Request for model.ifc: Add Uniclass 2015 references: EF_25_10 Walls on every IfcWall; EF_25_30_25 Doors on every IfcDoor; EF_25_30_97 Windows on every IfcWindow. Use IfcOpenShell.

First a look at what the model holds.

```python
import ifcopenshell

model = ifcopenshell.open("model.ifc")
print(model.schema)
print("classifications:", [c.Name for c in model.by_type("IfcClassification")])
for ifc_class in ("IfcDoor", "IfcRoof", "IfcStair", "IfcWall", "IfcWindow"):
    print(ifc_class, len(model.by_type(ifc_class)))
```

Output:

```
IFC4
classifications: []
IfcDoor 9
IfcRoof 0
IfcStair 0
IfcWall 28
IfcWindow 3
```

```python
import ifcopenshell
import ifcopenshell.api.classification

model = ifcopenshell.open("model.ifc")

system = ifcopenshell.api.classification.add_classification(model, classification="Uniclass 2015")

codes = {
    "IfcWall": ("EF_25_10", "Walls"),
    "IfcDoor": ("EF_25_30_25", "Doors"),
    "IfcWindow": ("EF_25_30_97", "Windows"),
}
for ifc_class, (code, name) in codes.items():
    products = model.by_type(ifc_class)
    ifcopenshell.api.classification.add_reference(
        model, products=products, classification=system, identification=code, name=name
    )
    print(code, len(products))

model.write("model_updated.ifc")
```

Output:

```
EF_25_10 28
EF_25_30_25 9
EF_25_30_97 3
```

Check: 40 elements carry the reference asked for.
